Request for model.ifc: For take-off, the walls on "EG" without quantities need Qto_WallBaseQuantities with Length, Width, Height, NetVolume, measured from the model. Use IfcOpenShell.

First a look at what the model holds.

```python
import ifcopenshell
import ifcopenshell.util.element
import ifcopenshell.util.unit

model = ifcopenshell.open("model.ifc")
print(model.schema)
for unit_type in ("LENGTHUNIT", "AREAUNIT", "VOLUMEUNIT"):
    print(unit_type, ifcopenshell.util.unit.calculate_unit_scale(model, unit_type))
storey = next(s for s in model.by_type("IfcBuildingStorey") if s.Name == "EG")
walls = [e for e in ifcopenshell.util.element.get_decomposition(storey) if e.is_a("IfcWall")]
for e in sorted(walls, key=lambda e: e.id()):
    print(e.id(), e.is_a(), e.Name, list(ifcopenshell.util.element.get_psets(e, qtos_only=True)), sep=" | ")
```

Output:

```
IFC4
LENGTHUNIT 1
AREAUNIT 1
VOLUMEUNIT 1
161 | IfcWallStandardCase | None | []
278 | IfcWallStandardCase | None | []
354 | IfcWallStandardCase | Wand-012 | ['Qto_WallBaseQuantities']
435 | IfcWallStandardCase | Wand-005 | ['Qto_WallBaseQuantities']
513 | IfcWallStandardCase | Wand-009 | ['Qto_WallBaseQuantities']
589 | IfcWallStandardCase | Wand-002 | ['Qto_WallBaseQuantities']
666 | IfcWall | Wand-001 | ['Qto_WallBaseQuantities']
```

```python
import ifcopenshell
import ifcopenshell.api.pset
import ifcopenshell.geom
import ifcopenshell.util.element
import ifcopenshell.util.shape
import ifcopenshell.util.unit

model = ifcopenshell.open("model.ifc")
unit_scale = ifcopenshell.util.unit.calculate_unit_scale(model)
volume_scale = ifcopenshell.util.unit.calculate_unit_scale(model, "VOLUMEUNIT")
settings = ifcopenshell.geom.settings()

storey = next(s for s in model.by_type("IfcBuildingStorey") if s.Name == "EG")
walls = [e for e in ifcopenshell.util.element.get_decomposition(storey) if e.is_a("IfcWall")]

for e in sorted(walls, key=lambda e: e.id()):
    if ifcopenshell.util.element.get_psets(e, qtos_only=True, should_inherit=False):
        continue
    # Geometry comes back in metres, in the element's own axes.
    shape = ifcopenshell.geom.create_shape(settings, e)
    values = {
        "Length": ifcopenshell.util.shape.get_x(shape.geometry) / unit_scale,
        "Width": ifcopenshell.util.shape.get_y(shape.geometry) / unit_scale,
        "Height": ifcopenshell.util.shape.get_z(shape.geometry) / unit_scale,
        "NetVolume": ifcopenshell.util.shape.get_volume(shape.geometry) / volume_scale,
    }
    qto = ifcopenshell.api.pset.add_qto(model, product=e, name="Qto_WallBaseQuantities")
    ifcopenshell.api.pset.edit_qto(model, qto=qto, properties=values)
    print(e.id(), {k: round(v, 3) for k, v in values.items()})

model.write("model_updated.ifc")
```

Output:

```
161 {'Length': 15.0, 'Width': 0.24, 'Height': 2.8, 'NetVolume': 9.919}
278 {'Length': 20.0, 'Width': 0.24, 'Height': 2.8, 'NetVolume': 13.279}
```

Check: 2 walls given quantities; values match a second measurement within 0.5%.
